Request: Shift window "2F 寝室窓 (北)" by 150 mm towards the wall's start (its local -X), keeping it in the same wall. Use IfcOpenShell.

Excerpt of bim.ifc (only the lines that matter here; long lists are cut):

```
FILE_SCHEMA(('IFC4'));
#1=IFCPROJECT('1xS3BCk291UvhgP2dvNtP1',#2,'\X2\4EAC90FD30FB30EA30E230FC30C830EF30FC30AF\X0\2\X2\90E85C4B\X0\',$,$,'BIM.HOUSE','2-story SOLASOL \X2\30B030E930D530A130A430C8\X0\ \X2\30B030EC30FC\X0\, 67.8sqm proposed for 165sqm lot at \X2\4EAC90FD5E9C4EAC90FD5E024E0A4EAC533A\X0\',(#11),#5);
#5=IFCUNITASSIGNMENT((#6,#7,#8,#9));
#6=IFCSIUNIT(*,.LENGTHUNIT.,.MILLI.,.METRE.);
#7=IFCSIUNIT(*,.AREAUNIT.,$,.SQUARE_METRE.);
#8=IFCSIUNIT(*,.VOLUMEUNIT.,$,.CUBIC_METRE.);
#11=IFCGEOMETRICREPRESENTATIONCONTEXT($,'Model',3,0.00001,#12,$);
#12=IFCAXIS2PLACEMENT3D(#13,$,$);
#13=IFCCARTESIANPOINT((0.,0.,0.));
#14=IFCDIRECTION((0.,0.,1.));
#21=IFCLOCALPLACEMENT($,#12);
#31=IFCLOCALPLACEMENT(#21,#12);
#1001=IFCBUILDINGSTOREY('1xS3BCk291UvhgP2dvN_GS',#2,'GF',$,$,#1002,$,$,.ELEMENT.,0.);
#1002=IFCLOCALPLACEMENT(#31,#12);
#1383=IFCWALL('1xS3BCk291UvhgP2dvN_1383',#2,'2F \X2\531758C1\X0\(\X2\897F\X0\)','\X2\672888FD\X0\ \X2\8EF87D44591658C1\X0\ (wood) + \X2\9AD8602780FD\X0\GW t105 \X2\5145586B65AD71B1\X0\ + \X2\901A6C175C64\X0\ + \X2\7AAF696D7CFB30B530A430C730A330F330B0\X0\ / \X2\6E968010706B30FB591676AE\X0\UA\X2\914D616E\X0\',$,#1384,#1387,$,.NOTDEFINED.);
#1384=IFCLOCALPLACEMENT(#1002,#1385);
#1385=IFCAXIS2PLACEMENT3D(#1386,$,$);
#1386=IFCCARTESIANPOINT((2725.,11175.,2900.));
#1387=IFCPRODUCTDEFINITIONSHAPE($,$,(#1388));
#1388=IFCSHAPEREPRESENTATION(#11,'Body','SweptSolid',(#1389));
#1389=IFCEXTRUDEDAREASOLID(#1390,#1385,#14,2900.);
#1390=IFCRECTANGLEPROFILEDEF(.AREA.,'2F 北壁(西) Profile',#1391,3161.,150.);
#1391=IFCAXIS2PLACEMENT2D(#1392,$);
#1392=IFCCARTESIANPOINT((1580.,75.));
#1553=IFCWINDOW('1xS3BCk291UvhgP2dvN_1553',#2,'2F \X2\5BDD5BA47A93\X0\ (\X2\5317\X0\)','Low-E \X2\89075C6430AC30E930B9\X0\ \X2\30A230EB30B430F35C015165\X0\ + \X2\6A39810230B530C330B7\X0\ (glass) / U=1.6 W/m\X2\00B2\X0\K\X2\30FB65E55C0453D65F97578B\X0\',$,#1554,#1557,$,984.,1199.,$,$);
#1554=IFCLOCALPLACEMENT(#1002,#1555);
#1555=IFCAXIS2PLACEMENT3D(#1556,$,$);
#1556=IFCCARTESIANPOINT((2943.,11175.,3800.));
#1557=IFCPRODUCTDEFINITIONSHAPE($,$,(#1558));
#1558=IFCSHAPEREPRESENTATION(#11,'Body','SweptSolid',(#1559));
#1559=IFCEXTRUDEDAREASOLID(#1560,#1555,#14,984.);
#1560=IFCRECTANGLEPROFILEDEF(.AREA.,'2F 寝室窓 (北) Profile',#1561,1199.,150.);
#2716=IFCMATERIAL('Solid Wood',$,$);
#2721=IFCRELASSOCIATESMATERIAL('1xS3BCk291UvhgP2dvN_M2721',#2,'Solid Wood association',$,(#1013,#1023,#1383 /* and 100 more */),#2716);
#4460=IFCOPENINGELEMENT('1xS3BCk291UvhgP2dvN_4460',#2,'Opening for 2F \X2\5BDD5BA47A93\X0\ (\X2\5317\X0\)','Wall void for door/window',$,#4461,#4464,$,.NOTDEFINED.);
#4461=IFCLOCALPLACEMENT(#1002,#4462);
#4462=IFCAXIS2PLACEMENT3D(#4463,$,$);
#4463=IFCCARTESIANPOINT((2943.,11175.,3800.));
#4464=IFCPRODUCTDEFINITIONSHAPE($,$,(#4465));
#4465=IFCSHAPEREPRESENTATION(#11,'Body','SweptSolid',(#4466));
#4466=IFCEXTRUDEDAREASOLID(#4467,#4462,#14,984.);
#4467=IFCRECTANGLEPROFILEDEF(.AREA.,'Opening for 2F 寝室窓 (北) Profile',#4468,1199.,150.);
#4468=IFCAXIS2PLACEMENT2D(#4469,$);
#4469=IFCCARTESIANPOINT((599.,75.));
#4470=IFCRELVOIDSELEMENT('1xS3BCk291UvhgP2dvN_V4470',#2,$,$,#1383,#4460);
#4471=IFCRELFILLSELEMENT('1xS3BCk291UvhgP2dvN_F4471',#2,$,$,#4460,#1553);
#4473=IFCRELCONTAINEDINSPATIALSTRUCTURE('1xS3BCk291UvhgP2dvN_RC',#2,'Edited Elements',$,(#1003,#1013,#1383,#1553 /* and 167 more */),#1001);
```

```python
import ifcopenshell
import ifcopenshell.api.geometry
import ifcopenshell.util.placement
import ifcopenshell.util.unit

model = ifcopenshell.open("bim.ifc")
unit_scale = ifcopenshell.util.unit.calculate_unit_scale(model)

window = model.by_guid("1xS3BCk291UvhgP2dvN_1553")
opening = window.FillsVoids[0].RelatingOpeningElement
wall = opening.VoidsElements[0].RelatingBuildingElement

wall_matrix = ifcopenshell.util.placement.get_local_placement(wall.ObjectPlacement)
shift = wall_matrix[:3, 0] * -0.15 / unit_scale
before = ifcopenshell.util.placement.get_local_placement(window.ObjectPlacement)[:3, 3].copy()

# The window is not placed relative to its opening, so move both.
for product in (opening, window):
    matrix = ifcopenshell.util.placement.get_local_placement(product.ObjectPlacement)
    matrix[:3, 3] += shift
    ifcopenshell.api.geometry.edit_object_placement(model, product=product, matrix=matrix, is_si=False)

after = ifcopenshell.util.placement.get_local_placement(window.ObjectPlacement)[:3, 3]
print("window moved by", (after - before).round(3) + 0.0)

model.write("bim_updated.ifc")
```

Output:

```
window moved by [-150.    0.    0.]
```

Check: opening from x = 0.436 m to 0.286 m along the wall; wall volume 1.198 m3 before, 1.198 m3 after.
